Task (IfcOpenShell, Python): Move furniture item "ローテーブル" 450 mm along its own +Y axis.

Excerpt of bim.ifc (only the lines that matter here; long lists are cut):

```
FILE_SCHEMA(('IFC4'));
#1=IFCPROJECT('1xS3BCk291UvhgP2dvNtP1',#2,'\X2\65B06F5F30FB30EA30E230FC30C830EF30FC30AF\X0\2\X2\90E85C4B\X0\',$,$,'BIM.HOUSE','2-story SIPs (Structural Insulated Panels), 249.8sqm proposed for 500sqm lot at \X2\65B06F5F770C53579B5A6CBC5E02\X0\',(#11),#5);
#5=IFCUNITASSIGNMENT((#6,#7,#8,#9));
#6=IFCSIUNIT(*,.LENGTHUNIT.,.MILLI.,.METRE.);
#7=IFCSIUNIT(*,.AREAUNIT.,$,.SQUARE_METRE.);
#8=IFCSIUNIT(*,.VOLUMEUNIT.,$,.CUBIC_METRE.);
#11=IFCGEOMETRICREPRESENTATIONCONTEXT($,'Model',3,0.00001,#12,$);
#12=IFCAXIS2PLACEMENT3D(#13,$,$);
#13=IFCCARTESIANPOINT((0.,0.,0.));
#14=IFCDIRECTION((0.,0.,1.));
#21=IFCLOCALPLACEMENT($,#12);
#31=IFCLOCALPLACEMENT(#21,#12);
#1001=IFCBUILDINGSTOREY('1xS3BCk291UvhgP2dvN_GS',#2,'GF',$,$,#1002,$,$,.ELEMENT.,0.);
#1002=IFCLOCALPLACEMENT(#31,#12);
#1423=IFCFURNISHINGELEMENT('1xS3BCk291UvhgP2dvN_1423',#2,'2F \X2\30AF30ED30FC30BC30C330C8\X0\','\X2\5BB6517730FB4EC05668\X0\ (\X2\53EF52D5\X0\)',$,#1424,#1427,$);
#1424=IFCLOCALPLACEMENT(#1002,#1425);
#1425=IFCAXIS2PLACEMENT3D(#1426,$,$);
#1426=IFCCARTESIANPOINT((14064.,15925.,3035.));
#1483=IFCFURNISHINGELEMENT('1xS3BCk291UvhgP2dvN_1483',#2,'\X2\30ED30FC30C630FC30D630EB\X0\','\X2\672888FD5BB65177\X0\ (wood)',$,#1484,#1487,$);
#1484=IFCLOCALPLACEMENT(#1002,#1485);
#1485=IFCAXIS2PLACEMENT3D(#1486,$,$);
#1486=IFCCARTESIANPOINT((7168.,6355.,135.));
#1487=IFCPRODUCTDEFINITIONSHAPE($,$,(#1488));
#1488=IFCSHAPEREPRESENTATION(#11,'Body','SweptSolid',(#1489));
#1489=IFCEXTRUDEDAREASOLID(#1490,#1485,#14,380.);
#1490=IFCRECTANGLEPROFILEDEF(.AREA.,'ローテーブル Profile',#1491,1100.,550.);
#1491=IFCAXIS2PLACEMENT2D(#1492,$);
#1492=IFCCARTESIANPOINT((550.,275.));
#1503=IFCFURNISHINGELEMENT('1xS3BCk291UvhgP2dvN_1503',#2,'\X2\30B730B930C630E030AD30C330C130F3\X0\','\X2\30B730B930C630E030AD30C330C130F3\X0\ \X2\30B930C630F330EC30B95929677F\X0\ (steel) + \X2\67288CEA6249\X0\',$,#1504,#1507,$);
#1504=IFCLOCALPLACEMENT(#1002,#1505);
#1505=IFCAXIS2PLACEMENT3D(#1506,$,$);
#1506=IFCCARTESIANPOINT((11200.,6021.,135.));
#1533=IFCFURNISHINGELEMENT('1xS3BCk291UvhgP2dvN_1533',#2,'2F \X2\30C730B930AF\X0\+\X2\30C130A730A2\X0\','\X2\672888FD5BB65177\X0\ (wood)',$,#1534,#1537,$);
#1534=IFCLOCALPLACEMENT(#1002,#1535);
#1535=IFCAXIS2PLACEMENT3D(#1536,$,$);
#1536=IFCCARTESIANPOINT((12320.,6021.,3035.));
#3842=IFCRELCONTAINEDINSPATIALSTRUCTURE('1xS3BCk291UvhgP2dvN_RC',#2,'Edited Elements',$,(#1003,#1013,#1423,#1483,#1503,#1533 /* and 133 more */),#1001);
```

```python
import ifcopenshell
import ifcopenshell.api.geometry
import ifcopenshell.util.placement

model = ifcopenshell.open("bim.ifc")

item = model.by_id(1483)
matrix = ifcopenshell.util.placement.get_local_placement(item.ObjectPlacement)
matrix[:3, 3] += matrix[:3, 1] * 450.0
ifcopenshell.api.geometry.edit_object_placement(model, product=item, matrix=matrix, is_si=False)

print(ifcopenshell.util.placement.get_local_placement(item.ObjectPlacement).round(3) + 0.0)

model.write("bim_updated.ifc")
```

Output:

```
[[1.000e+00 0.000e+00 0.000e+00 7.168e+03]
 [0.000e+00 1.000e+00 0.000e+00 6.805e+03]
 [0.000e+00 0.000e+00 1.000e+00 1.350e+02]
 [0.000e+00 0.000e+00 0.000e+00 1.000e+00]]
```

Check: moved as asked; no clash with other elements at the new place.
